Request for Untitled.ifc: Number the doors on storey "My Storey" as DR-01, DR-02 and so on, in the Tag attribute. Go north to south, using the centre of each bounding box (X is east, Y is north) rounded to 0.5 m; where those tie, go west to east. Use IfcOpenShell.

First a look at what the model holds.

```python
import ifcopenshell
import ifcopenshell.util.element
import ifcopenshell.util.placement

model = ifcopenshell.open("Untitled.ifc")
print(model.schema)
storey = next(s for s in model.by_type("IfcBuildingStorey") if s.Name == "My Storey")
doors = [e for e in ifcopenshell.util.element.get_decomposition(storey) if e.is_a("IfcDoor")]
for e in sorted(doors, key=lambda e: e.id()):
    origin = ifcopenshell.util.placement.get_local_placement(e.ObjectPlacement)[:3, 3]
    print(e.id(), e.Tag, e.Name, origin.round(2) + 0.0, sep=" | ")
```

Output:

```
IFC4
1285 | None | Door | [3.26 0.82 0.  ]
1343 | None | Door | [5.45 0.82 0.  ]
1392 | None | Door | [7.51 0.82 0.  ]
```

```python
import ifcopenshell
import ifcopenshell.geom
import ifcopenshell.util.element
import ifcopenshell.util.shape

model = ifcopenshell.open("Untitled.ifc")
settings = ifcopenshell.geom.settings()
settings.set("use-world-coords", True)


def centre(element):
    shape = ifcopenshell.geom.create_shape(settings, element)
    return ifcopenshell.util.shape.get_bbox_centroid(shape.geometry)


storey = next(s for s in model.by_type("IfcBuildingStorey") if s.Name == "My Storey")
doors = [e for e in ifcopenshell.util.element.get_decomposition(storey) if e.is_a("IfcDoor")]

# Insertion points can sit at a corner or the storey origin, so sort by the geometry (in metres).
centres = {e: centre(e) for e in doors}
doors.sort(key=lambda e: (-round(centres[e][1] / 0.5), centres[e][0]))

for i, e in enumerate(doors, start=1):
    number = f"DR-{i:02d}"
    e.Tag = number
    print(e.id(), number)

model.write("Untitled_rev.ifc")
```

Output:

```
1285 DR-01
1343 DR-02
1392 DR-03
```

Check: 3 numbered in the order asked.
